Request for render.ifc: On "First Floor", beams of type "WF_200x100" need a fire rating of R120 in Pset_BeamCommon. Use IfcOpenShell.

First a look at what the model holds.

```python
import ifcopenshell
import ifcopenshell.util.element

model = ifcopenshell.open("render.ifc")
print(model.schema)
storey = next(s for s in model.by_type("IfcBuildingStorey") if s.Name == "First Floor")
beams = [e for e in ifcopenshell.util.element.get_decomposition(storey) if e.is_a("IfcBeam")]
seen = {}
for e in beams:
    element_type = ifcopenshell.util.element.get_type(e)
    key = (element_type.Name if element_type != e and element_type else None, ifcopenshell.util.element.get_pset(e, "Pset_BeamCommon", "FireRating"))
    seen[key] = seen.get(key, 0) + 1
for (name, value), count in sorted(seen.items(), key=str):
    print(count, "x", name, "|", value)
```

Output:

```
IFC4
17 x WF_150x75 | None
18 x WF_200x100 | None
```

```python
import ifcopenshell
import ifcopenshell.api.pset
import ifcopenshell.util.element

model = ifcopenshell.open("render.ifc")

storey = next(s for s in model.by_type("IfcBuildingStorey") if s.Name == "First Floor")
beams = [e for e in ifcopenshell.util.element.get_decomposition(storey) if e.is_a("IfcBeam")]

count = 0
for e in beams:
    element_type = ifcopenshell.util.element.get_type(e)
    if element_type in (None, e) or element_type.Name != "WF_200x100":
        continue
    # add_pset returns the element's existing set when there is one.
    pset = ifcopenshell.api.pset.add_pset(model, product=e, name="Pset_BeamCommon")
    ifcopenshell.api.pset.edit_pset(model, pset=pset, properties={"FireRating": "R120"})
    count += 1

print(count, "beams updated")

model.write("render-out.ifc")
```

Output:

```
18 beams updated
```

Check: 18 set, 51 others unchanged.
